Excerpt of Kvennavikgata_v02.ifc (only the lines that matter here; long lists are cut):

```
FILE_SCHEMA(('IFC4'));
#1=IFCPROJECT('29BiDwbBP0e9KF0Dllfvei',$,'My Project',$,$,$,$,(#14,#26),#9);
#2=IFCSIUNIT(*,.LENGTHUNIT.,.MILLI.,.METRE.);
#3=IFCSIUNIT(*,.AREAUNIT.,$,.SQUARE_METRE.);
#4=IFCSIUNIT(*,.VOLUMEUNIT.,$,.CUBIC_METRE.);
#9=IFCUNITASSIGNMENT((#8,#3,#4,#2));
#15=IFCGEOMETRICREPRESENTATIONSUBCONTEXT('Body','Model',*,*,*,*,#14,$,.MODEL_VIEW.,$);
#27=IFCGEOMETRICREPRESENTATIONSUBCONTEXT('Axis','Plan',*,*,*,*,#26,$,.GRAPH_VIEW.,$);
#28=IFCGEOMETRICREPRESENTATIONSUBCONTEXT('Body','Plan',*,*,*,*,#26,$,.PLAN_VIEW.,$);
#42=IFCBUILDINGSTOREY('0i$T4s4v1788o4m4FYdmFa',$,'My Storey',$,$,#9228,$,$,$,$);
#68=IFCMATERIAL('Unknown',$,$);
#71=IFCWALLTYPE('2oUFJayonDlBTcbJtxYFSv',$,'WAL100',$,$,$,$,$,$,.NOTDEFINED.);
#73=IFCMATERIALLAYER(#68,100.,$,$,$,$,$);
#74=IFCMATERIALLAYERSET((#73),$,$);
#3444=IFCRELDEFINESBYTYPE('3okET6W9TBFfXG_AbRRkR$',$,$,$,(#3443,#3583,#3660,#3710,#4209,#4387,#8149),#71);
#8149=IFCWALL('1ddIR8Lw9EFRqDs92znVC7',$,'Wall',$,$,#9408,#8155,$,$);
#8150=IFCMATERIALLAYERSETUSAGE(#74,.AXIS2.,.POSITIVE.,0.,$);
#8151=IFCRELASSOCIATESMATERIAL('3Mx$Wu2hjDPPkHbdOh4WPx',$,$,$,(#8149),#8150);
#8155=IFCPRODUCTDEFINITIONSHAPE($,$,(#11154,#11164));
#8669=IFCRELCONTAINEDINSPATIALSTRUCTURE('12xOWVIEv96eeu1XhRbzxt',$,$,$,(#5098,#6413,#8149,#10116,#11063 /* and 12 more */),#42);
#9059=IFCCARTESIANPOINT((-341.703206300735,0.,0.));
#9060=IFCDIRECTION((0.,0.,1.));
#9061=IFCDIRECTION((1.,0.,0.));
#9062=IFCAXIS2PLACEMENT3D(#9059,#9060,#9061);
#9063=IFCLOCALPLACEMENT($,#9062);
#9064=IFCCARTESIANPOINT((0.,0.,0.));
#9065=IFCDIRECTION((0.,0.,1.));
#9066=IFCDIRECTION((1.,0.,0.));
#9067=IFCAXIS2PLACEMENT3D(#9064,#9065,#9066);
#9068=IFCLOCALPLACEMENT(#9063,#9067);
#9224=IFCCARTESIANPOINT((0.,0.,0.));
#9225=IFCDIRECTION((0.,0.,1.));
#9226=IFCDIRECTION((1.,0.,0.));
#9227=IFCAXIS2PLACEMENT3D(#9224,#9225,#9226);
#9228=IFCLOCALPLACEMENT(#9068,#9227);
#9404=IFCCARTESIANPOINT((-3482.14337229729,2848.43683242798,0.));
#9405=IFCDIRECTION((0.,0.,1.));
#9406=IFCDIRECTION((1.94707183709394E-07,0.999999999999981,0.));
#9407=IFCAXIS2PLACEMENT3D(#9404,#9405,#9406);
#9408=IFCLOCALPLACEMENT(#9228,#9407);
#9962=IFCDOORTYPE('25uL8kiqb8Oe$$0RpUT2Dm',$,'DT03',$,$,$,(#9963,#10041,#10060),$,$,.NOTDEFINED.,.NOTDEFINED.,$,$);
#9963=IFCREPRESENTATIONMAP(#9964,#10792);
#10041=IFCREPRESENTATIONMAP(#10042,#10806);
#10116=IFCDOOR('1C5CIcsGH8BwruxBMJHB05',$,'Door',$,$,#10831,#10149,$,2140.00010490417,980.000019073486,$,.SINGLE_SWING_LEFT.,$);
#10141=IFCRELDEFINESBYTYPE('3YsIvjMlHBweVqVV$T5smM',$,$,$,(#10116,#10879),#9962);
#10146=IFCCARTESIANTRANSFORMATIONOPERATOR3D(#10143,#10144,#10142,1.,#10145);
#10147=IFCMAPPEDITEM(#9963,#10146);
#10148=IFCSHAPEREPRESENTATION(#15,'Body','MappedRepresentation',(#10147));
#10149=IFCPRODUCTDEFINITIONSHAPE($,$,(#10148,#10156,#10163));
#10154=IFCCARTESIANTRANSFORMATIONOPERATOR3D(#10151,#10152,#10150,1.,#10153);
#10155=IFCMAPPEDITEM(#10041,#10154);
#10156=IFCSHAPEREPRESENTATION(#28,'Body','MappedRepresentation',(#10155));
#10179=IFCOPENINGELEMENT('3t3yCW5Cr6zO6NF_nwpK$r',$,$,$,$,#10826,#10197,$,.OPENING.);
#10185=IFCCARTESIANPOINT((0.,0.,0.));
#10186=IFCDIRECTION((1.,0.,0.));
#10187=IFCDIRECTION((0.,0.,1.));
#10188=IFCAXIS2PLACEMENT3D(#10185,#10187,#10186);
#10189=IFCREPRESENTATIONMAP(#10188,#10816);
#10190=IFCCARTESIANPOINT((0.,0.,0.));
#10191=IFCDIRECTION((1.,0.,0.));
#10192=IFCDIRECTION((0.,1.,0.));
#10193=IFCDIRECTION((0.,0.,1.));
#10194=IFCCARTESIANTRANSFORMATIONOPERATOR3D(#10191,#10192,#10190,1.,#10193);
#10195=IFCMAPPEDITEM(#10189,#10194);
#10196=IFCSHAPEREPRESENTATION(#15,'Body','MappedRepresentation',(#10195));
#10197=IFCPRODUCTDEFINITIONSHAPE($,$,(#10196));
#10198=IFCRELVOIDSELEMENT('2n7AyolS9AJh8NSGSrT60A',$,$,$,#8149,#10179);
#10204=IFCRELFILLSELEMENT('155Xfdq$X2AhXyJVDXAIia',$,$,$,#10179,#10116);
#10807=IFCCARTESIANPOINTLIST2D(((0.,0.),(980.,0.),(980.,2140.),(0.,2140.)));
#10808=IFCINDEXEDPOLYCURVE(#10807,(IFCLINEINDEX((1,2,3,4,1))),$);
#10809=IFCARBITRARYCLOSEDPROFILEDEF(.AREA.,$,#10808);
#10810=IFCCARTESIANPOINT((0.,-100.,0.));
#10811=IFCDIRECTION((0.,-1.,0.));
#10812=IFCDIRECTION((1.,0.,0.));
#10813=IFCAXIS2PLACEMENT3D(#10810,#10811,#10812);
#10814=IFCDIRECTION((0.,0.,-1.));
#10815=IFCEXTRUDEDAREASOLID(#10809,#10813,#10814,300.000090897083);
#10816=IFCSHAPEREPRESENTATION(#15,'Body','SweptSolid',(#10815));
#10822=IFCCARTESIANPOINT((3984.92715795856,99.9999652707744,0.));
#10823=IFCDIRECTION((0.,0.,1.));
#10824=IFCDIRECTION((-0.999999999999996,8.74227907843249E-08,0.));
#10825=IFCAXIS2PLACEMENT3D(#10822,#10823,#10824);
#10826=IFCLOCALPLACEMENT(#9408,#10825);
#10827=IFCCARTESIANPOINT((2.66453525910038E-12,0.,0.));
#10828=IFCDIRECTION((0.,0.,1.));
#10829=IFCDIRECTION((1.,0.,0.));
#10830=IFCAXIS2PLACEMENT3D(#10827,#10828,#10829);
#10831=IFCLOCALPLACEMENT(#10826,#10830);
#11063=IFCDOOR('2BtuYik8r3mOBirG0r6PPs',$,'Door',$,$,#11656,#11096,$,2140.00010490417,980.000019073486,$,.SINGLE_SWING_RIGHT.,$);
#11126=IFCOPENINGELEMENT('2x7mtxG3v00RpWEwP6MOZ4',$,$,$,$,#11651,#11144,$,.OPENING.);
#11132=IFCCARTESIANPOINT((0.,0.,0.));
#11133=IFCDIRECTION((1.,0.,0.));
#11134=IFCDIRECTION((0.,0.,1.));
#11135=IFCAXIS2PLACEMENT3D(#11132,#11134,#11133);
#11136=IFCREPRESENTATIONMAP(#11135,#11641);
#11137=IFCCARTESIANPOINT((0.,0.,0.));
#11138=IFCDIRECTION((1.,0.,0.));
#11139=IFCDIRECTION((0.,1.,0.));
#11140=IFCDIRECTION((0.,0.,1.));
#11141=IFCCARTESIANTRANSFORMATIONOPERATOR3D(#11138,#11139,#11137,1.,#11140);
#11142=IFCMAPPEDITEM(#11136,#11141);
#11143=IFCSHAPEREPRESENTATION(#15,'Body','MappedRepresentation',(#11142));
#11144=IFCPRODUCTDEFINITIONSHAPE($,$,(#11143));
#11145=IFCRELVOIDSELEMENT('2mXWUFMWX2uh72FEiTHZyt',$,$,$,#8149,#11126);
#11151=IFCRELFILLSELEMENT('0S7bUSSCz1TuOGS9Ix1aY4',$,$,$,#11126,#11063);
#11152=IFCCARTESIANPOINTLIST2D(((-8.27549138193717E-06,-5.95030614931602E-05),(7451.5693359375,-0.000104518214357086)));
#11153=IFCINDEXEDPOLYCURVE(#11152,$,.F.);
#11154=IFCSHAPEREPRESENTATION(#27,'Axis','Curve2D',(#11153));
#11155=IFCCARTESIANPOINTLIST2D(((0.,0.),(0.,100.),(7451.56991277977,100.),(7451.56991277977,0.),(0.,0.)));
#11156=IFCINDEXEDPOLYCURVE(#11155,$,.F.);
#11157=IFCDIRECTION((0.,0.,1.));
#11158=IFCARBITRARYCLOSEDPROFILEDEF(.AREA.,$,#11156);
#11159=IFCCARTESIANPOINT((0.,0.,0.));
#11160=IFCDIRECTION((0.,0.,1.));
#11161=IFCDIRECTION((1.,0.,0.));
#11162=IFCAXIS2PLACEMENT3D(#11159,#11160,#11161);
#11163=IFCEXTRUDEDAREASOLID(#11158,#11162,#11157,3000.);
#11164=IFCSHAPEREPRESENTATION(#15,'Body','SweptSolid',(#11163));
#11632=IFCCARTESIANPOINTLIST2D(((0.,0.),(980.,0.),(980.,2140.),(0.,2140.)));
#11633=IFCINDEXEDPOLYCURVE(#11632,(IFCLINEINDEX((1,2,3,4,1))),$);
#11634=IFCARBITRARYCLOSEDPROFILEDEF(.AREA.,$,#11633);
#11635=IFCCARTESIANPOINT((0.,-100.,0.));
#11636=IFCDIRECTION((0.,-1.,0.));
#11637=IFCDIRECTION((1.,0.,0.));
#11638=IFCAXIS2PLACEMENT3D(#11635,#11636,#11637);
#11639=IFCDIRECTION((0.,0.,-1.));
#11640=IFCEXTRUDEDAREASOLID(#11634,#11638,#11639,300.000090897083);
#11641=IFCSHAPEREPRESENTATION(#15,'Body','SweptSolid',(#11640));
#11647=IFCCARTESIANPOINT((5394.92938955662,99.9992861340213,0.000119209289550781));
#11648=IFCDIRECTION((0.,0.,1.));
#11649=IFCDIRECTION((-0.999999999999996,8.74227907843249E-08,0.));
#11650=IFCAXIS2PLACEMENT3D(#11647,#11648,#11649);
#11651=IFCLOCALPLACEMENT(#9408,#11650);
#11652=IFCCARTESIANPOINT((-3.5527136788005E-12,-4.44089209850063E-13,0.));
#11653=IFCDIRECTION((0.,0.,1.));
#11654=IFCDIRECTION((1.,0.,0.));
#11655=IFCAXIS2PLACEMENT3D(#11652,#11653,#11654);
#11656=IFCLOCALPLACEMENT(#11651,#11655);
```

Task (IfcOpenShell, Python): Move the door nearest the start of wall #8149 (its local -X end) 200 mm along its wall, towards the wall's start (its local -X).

```python
import ifcopenshell
import ifcopenshell.api.geometry
import ifcopenshell.util.placement
import ifcopenshell.util.unit

model = ifcopenshell.open("Kvennavikgata_v02.ifc")
unit_scale = ifcopenshell.util.unit.calculate_unit_scale(model)

door = model.by_guid("1C5CIcsGH8BwruxBMJHB05")
opening = door.FillsVoids[0].RelatingOpeningElement
wall = opening.VoidsElements[0].RelatingBuildingElement

wall_matrix = ifcopenshell.util.placement.get_local_placement(wall.ObjectPlacement)
shift = wall_matrix[:3, 0] * -0.2 / unit_scale
before = ifcopenshell.util.placement.get_local_placement(door.ObjectPlacement)[:3, 3].copy()

# The door is placed relative to its opening, so it follows when the opening moves.
matrix = ifcopenshell.util.placement.get_local_placement(opening.ObjectPlacement)
matrix[:3, 3] += shift
ifcopenshell.api.geometry.edit_object_placement(
    model, product=opening, matrix=matrix, is_si=False, should_transform_children=True
)

after = ifcopenshell.util.placement.get_local_placement(door.ObjectPlacement)[:3, 3]
print("door moved by", (after - before).round(3) + 0.0)

model.write("Kvennavikgata_v02_v2.ifc")
```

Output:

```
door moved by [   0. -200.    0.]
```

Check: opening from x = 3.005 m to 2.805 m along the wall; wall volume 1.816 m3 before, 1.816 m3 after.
